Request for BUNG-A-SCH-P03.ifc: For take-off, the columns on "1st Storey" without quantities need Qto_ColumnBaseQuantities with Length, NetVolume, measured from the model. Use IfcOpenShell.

First a look at what the model holds.

```python
import ifcopenshell
import ifcopenshell.util.element
import ifcopenshell.util.unit

model = ifcopenshell.open("BUNG-A-SCH-P03.ifc")
print(model.schema)
for unit_type in ("LENGTHUNIT", "AREAUNIT", "VOLUMEUNIT"):
    print(unit_type, ifcopenshell.util.unit.calculate_unit_scale(model, unit_type))
storey = next(s for s in model.by_type("IfcBuildingStorey") if s.Name == "1st Storey")
columns = [e for e in ifcopenshell.util.element.get_decomposition(storey) if e.is_a("IfcColumn")]
for e in sorted(columns, key=lambda e: e.id()):
    print(e.id(), e.is_a(), e.Name, list(ifcopenshell.util.element.get_psets(e, qtos_only=True)), sep=" | ")
```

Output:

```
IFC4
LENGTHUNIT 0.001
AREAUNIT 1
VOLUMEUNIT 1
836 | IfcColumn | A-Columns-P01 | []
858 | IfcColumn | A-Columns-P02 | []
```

```python
import ifcopenshell
import ifcopenshell.api.pset
import ifcopenshell.geom
import ifcopenshell.util.element
import ifcopenshell.util.shape
import ifcopenshell.util.unit

model = ifcopenshell.open("BUNG-A-SCH-P03.ifc")
unit_scale = ifcopenshell.util.unit.calculate_unit_scale(model)
volume_scale = ifcopenshell.util.unit.calculate_unit_scale(model, "VOLUMEUNIT")
settings = ifcopenshell.geom.settings()

storey = next(s for s in model.by_type("IfcBuildingStorey") if s.Name == "1st Storey")
columns = [e for e in ifcopenshell.util.element.get_decomposition(storey) if e.is_a("IfcColumn")]

for e in sorted(columns, key=lambda e: e.id()):
    if ifcopenshell.util.element.get_psets(e, qtos_only=True, should_inherit=False):
        continue
    # Geometry comes back in metres, in the element's own axes.
    shape = ifcopenshell.geom.create_shape(settings, e)
    values = {
        "Length": ifcopenshell.util.shape.get_z(shape.geometry) / unit_scale,
        "NetVolume": ifcopenshell.util.shape.get_volume(shape.geometry) / volume_scale,
    }
    qto = ifcopenshell.api.pset.add_qto(model, product=e, name="Qto_ColumnBaseQuantities")
    ifcopenshell.api.pset.edit_qto(model, qto=qto, properties=values)
    print(e.id(), {k: round(v, 3) for k, v in values.items()})

model.write("BUNG-A-SCH-P03_rev.ifc")
```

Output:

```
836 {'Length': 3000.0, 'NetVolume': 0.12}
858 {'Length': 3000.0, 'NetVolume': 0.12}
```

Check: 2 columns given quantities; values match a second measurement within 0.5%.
